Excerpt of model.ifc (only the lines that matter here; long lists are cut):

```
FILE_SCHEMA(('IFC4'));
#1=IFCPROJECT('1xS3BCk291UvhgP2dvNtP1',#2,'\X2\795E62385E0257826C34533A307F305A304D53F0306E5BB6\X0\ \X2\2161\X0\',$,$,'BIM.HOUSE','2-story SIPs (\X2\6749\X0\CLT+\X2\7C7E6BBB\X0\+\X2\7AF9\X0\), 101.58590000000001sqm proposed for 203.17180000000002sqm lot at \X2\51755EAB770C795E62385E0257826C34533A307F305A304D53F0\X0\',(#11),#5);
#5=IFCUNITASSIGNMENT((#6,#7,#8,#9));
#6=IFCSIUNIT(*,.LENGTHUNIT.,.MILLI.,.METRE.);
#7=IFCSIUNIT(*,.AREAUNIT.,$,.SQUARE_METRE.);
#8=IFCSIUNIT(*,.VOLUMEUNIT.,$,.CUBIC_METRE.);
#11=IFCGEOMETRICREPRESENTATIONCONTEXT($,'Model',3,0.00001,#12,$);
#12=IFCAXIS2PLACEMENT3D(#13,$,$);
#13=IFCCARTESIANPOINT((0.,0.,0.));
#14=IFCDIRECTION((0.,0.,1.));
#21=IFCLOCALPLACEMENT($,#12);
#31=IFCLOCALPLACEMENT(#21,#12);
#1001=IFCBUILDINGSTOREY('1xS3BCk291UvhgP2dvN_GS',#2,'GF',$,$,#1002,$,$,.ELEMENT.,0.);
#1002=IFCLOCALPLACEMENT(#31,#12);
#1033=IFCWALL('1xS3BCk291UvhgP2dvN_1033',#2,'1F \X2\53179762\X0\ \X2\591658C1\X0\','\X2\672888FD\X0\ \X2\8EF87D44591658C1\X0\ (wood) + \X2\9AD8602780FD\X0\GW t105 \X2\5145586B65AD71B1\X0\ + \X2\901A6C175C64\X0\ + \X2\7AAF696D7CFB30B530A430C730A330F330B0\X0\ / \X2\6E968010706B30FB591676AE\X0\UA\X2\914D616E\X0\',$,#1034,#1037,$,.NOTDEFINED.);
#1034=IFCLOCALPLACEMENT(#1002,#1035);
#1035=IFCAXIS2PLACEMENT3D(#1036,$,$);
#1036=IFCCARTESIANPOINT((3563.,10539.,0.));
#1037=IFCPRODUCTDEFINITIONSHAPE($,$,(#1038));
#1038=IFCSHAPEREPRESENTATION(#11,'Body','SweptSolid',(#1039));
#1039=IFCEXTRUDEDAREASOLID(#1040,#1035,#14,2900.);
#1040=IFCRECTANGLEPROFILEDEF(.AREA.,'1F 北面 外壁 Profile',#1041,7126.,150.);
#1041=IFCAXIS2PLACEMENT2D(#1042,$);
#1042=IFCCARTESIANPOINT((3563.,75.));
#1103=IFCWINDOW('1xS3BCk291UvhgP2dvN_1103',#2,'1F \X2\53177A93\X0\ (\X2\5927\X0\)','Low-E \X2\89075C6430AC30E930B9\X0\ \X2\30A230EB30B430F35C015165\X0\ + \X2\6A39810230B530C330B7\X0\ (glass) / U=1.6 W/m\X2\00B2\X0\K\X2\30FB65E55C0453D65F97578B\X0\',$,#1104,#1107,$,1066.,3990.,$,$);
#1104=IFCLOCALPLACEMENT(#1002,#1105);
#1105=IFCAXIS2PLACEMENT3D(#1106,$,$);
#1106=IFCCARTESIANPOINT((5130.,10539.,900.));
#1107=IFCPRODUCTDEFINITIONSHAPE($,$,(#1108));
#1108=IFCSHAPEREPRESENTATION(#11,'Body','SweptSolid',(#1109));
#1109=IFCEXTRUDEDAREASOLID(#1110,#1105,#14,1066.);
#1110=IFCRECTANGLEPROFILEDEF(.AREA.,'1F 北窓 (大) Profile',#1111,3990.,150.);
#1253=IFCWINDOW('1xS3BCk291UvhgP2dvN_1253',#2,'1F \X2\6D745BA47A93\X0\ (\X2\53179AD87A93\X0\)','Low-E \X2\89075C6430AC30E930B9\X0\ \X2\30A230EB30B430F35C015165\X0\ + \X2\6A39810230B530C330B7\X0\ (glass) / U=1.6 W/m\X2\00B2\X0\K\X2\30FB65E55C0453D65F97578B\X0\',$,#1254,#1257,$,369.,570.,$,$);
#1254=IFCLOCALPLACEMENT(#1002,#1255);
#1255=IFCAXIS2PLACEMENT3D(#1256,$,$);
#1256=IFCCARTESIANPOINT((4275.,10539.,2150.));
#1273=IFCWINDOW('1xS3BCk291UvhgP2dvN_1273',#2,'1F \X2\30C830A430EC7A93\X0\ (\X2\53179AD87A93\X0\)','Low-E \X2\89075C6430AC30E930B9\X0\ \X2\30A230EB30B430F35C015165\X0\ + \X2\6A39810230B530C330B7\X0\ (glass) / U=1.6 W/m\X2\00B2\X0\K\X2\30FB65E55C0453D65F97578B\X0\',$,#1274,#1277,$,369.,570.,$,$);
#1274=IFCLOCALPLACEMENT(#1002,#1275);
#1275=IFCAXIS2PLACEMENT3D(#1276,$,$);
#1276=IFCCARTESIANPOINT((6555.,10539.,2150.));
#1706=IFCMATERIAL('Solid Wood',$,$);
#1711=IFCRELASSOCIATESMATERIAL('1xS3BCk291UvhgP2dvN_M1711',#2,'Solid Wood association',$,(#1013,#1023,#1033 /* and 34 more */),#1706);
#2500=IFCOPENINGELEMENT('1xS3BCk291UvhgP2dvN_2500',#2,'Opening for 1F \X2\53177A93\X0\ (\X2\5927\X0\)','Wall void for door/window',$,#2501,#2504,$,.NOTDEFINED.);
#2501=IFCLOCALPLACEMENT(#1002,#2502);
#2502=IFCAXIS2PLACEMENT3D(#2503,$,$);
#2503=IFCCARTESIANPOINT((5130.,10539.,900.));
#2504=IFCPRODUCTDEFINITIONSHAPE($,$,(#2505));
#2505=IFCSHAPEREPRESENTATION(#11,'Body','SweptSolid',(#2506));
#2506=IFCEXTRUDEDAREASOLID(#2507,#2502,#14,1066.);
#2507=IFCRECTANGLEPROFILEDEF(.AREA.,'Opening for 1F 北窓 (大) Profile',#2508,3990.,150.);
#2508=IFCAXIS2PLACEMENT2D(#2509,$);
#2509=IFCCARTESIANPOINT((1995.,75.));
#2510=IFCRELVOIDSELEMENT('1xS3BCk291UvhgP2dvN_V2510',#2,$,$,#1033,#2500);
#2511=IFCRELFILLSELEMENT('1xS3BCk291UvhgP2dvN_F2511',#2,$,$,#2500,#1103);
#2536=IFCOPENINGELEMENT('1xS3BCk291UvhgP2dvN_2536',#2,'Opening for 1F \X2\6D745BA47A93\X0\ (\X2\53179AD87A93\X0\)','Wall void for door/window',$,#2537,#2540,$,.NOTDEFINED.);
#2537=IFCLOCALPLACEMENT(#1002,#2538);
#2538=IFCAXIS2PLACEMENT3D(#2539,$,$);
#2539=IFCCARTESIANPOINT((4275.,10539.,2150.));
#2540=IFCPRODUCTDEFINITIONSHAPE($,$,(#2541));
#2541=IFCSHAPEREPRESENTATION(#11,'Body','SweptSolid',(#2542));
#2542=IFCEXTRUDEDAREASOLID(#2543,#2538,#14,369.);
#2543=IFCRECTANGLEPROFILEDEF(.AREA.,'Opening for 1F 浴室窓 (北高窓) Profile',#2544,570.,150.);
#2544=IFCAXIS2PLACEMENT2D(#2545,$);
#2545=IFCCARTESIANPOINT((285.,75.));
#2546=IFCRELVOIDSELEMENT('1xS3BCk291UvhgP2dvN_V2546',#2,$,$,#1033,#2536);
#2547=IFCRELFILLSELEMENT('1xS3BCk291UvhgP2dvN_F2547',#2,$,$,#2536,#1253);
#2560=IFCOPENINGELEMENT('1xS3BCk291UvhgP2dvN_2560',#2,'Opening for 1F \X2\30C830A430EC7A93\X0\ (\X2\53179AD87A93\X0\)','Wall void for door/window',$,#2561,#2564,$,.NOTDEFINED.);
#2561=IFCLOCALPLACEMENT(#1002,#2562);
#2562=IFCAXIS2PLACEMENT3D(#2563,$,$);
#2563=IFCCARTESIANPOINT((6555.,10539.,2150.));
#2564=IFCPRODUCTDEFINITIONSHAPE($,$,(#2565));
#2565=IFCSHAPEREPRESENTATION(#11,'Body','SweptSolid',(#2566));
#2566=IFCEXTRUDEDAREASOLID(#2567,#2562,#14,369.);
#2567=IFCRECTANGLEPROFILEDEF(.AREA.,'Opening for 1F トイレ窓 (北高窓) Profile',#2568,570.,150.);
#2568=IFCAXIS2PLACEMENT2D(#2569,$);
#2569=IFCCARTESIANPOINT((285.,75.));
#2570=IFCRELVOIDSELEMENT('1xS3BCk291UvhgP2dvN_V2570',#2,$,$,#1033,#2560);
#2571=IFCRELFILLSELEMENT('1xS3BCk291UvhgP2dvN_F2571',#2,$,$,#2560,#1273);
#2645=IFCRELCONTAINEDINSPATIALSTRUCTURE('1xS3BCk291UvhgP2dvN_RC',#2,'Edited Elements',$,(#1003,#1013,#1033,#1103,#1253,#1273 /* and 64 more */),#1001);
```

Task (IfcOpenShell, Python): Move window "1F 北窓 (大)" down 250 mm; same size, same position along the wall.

```python
import numpy as np
import ifcopenshell
import ifcopenshell.api.geometry
import ifcopenshell.util.placement
import ifcopenshell.util.unit

model = ifcopenshell.open("model.ifc")
unit_scale = ifcopenshell.util.unit.calculate_unit_scale(model)

window = model.by_guid("1xS3BCk291UvhgP2dvN_1103")
opening = window.FillsVoids[0].RelatingOpeningElement
dz = -0.25 / unit_scale

shift = np.array([0.0, 0.0, dz])
# The window is not placed relative to its opening, so move both.
for product in (opening, window):
    matrix = ifcopenshell.util.placement.get_local_placement(product.ObjectPlacement)
    matrix[:3, 3] += shift
    ifcopenshell.api.geometry.edit_object_placement(model, product=product, matrix=matrix, is_si=False)

print(f"moved by {dz * unit_scale:+.3f} m")

model.write("model-out.ifc")
```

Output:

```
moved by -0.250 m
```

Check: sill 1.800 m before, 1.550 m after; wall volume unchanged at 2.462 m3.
